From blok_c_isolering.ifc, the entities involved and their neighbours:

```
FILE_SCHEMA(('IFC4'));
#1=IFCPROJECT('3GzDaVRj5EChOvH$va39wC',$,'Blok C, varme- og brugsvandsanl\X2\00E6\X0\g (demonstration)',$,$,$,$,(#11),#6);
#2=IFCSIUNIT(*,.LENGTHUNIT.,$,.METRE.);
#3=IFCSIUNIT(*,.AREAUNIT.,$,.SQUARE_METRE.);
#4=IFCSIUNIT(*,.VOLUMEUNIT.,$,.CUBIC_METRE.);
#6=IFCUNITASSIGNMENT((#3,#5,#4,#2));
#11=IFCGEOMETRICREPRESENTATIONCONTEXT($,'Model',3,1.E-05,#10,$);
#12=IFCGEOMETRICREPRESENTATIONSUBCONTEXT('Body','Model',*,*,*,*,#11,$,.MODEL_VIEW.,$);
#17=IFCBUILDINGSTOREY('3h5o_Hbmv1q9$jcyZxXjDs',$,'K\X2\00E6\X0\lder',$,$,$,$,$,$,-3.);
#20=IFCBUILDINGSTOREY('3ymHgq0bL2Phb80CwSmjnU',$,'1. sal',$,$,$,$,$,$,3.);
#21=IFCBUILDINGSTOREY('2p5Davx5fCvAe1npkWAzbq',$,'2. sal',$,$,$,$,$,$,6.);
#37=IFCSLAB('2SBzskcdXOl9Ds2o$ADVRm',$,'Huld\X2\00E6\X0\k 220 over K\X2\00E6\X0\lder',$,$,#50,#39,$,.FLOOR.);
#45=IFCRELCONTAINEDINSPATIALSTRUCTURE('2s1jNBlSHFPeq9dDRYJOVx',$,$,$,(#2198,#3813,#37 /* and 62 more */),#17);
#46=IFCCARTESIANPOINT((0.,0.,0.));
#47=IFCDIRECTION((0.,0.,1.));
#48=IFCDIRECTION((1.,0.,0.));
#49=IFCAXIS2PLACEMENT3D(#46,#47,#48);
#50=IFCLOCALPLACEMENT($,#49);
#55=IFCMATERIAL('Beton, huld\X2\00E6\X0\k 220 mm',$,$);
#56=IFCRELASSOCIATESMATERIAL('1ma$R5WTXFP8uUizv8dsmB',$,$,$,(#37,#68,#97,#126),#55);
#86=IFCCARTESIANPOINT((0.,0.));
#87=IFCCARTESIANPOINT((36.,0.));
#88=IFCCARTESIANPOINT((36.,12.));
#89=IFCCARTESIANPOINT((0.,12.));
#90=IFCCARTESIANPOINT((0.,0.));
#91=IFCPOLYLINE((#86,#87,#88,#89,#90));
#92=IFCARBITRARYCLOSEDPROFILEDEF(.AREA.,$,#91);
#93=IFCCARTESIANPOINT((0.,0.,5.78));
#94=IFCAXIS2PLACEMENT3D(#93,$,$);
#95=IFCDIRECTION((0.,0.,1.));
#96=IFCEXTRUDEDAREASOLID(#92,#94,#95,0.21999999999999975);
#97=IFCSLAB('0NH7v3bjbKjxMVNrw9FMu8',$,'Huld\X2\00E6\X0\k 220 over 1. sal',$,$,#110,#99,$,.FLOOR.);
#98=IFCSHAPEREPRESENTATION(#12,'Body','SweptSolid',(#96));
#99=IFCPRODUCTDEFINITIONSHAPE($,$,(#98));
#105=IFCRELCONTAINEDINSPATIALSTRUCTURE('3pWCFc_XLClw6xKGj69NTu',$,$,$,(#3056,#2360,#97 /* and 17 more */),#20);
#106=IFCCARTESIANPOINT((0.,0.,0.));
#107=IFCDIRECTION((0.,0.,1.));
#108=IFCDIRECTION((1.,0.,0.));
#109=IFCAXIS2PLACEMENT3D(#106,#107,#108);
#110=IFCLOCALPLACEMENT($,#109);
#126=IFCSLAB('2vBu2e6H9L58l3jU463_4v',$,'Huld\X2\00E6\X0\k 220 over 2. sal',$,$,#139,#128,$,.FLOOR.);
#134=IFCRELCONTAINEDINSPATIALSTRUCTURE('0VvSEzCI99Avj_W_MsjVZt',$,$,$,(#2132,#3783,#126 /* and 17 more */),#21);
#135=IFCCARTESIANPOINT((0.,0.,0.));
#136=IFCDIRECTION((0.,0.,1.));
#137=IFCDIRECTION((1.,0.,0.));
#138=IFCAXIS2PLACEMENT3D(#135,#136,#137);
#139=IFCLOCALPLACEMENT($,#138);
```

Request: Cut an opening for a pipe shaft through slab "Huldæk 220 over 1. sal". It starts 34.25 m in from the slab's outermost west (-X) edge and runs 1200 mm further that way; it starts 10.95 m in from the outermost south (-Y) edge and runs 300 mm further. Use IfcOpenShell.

```python
import numpy as np
import ifcopenshell
import ifcopenshell.api.feature
import ifcopenshell.api.geometry
import ifcopenshell.api.root
import ifcopenshell.geom
import ifcopenshell.util.placement
import ifcopenshell.util.representation
import ifcopenshell.util.shape
import ifcopenshell.util.unit

model = ifcopenshell.open("blok_c_isolering.ifc")
unit_scale = ifcopenshell.util.unit.calculate_unit_scale(model)
settings = ifcopenshell.geom.settings()


def volume(element):
    """Net volume in cubic metres, openings subtracted."""
    shape = ifcopenshell.geom.create_shape(settings, element)
    return ifcopenshell.util.shape.get_volume(shape.geometry)


slab = model.by_guid("0NH7v3bjbKjxMVNrw9FMu8")
before = volume(slab)

# Extent in the slab's own axes, in metres. The edges named are its -X and -Y sides.
slab_shape = ifcopenshell.geom.create_shape(settings, slab)
vertices = ifcopenshell.util.shape.get_vertices(slab_shape.geometry)
x_min, y_min, bottom = vertices.min(axis=0)
top = vertices[:, 2].max()

opening = ifcopenshell.api.root.create_entity(model, ifc_class="IfcOpeningElement", name="Pipe shaft opening", predefined_type="OPENING")
context = ifcopenshell.util.representation.get_context(model, "Model", "Body", "MODEL_VIEW")
width, depth = 1.2, 0.3
outline = [(0.0, 0.0), (width, 0.0), (width, depth), (0.0, depth), (0.0, 0.0)]
# Overshoot both faces by 50 mm so the cut is clean.
shape = ifcopenshell.api.geometry.add_slab_representation(
    model, context=context, depth=top - bottom + 0.1, polyline=outline
)
ifcopenshell.api.geometry.assign_representation(model, product=opening, representation=shape)

matrix = ifcopenshell.util.placement.get_local_placement(slab.ObjectPlacement)
matrix[:, 3] = matrix @ np.append(np.array([x_min + 34.25, y_min + 10.95, bottom - 0.05]) / unit_scale, 1.0)
ifcopenshell.api.geometry.edit_object_placement(model, product=opening, matrix=matrix, is_si=False)
ifcopenshell.api.feature.add_feature(model, feature=opening, element=slab)

after = volume(slab)

print(f"slab volume {before:.3f} -> {after:.3f} m3")

model.write("blok_c_isolering_edited.ifc")
```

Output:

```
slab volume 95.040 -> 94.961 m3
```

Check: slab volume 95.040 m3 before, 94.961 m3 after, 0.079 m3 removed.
